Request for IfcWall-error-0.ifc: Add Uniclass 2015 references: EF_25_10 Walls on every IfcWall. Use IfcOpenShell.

First a look at what the model holds.

```python
import ifcopenshell

model = ifcopenshell.open("IfcWall-error-0.ifc")
print(model.schema)
print("classifications:", [c.Name for c in model.by_type("IfcClassification")])
for ifc_class in ("IfcDoor", "IfcRoof", "IfcStair", "IfcWall", "IfcWindow"):
    print(ifc_class, len(model.by_type(ifc_class)))
```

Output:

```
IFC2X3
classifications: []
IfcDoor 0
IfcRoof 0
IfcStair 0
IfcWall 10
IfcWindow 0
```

```python
import ifcopenshell
import ifcopenshell.api.classification

model = ifcopenshell.open("IfcWall-error-0.ifc")

# IFC2X3 requires Source and Edition and has no link from the project to the system.
system = model.create_entity("IfcClassification", Source="NBS", Edition="2015", Name="Uniclass 2015")

codes = {
    "IfcWall": ("EF_25_10", "Walls"),
}
for ifc_class, (code, name) in codes.items():
    products = model.by_type(ifc_class)
    ifcopenshell.api.classification.add_reference(
        model, products=products, classification=system, identification=code, name=name
    )
    print(code, len(products))

model.write("IfcWall-error-0_updated.ifc")
```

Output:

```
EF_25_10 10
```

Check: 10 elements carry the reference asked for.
